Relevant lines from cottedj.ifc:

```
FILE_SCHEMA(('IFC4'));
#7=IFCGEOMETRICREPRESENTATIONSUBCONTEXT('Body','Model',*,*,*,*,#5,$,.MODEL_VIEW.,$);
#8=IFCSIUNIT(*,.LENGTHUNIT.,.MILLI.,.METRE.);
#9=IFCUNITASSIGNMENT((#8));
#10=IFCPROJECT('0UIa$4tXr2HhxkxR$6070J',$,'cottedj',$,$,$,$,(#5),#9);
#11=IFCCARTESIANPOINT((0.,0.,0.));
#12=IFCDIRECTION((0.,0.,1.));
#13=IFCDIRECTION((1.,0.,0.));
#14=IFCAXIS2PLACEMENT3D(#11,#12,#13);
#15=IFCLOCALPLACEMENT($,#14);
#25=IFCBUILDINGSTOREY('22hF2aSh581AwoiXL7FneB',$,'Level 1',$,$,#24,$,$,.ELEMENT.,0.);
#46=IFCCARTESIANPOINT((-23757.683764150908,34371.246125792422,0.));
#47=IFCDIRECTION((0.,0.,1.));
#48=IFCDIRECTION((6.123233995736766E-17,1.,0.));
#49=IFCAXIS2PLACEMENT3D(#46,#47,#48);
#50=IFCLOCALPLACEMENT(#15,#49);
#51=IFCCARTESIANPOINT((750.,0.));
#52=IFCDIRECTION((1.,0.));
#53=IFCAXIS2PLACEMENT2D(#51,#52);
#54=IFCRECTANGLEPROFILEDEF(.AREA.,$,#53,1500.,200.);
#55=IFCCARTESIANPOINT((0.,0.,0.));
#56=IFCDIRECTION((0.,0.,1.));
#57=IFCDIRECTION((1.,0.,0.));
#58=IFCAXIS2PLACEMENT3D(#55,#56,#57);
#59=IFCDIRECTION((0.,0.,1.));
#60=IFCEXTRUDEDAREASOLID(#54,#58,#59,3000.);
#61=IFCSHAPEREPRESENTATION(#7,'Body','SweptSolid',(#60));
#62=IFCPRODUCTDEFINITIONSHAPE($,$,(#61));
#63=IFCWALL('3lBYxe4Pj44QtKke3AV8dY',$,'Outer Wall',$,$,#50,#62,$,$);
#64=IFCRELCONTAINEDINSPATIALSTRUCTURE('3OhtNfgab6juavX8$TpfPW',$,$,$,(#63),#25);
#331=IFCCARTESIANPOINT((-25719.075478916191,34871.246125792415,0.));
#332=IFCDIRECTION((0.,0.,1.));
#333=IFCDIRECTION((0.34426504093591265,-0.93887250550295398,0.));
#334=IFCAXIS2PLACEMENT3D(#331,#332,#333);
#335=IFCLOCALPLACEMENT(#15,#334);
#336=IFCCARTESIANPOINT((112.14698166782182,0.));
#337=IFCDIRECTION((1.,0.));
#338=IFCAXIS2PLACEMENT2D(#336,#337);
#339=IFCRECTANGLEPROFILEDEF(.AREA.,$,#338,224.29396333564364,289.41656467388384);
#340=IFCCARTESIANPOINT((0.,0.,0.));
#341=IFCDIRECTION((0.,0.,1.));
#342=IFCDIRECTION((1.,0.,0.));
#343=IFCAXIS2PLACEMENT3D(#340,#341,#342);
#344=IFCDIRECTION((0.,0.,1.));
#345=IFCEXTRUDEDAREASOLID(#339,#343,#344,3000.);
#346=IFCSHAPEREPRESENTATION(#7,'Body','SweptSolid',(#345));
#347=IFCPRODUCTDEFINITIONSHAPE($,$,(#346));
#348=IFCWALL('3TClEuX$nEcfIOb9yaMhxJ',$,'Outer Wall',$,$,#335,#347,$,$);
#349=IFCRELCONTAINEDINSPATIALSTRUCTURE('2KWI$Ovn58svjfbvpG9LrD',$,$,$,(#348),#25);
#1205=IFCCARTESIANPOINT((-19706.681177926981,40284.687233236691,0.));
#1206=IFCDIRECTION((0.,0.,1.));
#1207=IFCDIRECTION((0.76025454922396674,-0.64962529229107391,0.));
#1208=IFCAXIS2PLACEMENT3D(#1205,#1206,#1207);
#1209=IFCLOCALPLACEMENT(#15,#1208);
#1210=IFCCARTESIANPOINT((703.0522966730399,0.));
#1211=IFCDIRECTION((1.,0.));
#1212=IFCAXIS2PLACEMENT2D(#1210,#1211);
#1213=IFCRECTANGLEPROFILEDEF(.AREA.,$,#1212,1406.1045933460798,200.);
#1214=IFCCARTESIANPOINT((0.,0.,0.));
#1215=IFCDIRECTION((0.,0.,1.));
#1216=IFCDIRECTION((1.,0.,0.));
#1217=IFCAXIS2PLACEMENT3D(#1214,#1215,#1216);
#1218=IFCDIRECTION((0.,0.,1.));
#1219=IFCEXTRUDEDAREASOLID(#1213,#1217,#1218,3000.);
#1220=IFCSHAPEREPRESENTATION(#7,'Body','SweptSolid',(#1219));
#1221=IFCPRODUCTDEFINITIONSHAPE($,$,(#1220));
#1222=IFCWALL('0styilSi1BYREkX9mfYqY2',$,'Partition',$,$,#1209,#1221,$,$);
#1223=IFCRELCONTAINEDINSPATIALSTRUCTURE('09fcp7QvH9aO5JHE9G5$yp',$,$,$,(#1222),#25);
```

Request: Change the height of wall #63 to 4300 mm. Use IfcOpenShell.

```python
import ifcopenshell
import ifcopenshell.geom
import ifcopenshell.util.representation
import ifcopenshell.util.shape
import ifcopenshell.util.unit

model = ifcopenshell.open("cottedj.ifc")
unit_scale = ifcopenshell.util.unit.calculate_unit_scale(model)
settings = ifcopenshell.geom.settings()


def volume(element):
    """Net volume in cubic metres, openings subtracted."""
    shape = ifcopenshell.geom.create_shape(settings, element)
    return ifcopenshell.util.shape.get_volume(shape.geometry)


wall = model.by_guid("3lBYxe4Pj44QtKke3AV8dY")
before = volume(wall)

body = ifcopenshell.util.representation.get_representation(wall, "Model", "Body")
solid = body.Items[0]
old_height = solid.Depth
solid.Depth = 4.3 / unit_scale
after = volume(wall)

print(f"height {old_height:g} -> {solid.Depth:g}, volume {before:.3f} -> {after:.3f} m3")

model.write("cottedj_edited.ifc")
```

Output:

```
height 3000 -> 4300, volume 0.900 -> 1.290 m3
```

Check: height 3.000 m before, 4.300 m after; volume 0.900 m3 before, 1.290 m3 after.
